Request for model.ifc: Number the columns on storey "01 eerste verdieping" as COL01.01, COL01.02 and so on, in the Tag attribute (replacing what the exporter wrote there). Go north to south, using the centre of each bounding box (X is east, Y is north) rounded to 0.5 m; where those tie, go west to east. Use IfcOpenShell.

First a look at what the model holds.

```python
import ifcopenshell
import ifcopenshell.util.element
import ifcopenshell.util.placement

model = ifcopenshell.open("model.ifc")
print(model.schema)
storey = next(s for s in model.by_type("IfcBuildingStorey") if s.Name == "01 eerste verdieping")
columns = [e for e in ifcopenshell.util.element.get_decomposition(storey) if e.is_a("IfcColumn")]
for e in sorted(columns, key=lambda e: e.id()):
    origin = ifcopenshell.util.placement.get_local_placement(e.ObjectPlacement)[:3, 3]
    print(e.id(), e.Tag, e.Name, origin.round(2) + 0.0, sep=" | ")
```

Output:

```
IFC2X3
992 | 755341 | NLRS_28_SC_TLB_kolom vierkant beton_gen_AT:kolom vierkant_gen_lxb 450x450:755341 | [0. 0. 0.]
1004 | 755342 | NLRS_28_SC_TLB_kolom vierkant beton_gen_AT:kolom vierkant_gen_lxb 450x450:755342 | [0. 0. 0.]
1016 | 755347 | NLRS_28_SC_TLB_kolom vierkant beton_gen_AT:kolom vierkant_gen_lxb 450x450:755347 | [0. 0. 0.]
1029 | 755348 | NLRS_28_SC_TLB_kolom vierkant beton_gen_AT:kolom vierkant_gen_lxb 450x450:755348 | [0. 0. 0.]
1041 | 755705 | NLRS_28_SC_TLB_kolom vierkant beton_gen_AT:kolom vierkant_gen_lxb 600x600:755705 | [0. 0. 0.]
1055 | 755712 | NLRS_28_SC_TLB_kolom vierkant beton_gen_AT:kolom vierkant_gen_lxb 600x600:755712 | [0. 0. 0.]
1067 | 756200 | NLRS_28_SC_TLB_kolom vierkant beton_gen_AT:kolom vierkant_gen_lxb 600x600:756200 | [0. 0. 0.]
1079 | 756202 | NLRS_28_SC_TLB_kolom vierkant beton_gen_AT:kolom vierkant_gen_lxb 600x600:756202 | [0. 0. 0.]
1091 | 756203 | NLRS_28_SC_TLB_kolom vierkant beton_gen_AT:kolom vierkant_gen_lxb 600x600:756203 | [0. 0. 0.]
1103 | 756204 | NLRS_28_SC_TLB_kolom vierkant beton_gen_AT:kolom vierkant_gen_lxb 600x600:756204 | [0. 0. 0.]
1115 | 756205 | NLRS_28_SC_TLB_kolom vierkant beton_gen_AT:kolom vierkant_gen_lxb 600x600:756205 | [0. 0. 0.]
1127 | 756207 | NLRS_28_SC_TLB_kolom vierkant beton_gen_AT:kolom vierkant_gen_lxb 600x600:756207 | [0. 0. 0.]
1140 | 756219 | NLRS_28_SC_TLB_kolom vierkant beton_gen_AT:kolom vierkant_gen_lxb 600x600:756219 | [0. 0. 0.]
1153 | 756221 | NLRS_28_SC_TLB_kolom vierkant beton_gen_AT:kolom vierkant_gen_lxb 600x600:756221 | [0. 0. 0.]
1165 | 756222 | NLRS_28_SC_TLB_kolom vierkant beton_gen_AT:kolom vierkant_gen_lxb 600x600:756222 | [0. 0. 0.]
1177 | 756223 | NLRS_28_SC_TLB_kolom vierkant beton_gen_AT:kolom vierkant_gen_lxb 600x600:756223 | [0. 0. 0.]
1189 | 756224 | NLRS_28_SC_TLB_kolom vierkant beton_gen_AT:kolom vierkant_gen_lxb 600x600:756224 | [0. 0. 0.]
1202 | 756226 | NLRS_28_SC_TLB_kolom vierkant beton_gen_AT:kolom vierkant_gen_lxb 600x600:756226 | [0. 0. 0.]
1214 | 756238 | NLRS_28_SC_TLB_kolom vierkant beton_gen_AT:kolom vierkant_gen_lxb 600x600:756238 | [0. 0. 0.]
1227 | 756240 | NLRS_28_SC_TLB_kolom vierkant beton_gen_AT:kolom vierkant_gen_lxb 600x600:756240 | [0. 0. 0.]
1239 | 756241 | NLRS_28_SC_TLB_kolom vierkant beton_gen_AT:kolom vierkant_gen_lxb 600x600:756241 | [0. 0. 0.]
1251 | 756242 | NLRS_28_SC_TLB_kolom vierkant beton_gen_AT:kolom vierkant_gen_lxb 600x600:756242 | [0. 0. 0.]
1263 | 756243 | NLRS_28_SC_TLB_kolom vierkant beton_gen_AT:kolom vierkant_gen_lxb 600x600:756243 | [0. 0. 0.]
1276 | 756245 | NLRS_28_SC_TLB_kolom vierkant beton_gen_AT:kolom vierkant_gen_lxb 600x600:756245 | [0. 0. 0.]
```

```python
import ifcopenshell
import ifcopenshell.geom
import ifcopenshell.util.element
import ifcopenshell.util.shape

model = ifcopenshell.open("model.ifc")
settings = ifcopenshell.geom.settings()
settings.set("use-world-coords", True)


def centre(element):
    shape = ifcopenshell.geom.create_shape(settings, element)
    return ifcopenshell.util.shape.get_bbox_centroid(shape.geometry)


storey = next(s for s in model.by_type("IfcBuildingStorey") if s.Name == "01 eerste verdieping")
columns = [e for e in ifcopenshell.util.element.get_decomposition(storey) if e.is_a("IfcColumn")]

# Insertion points can sit at a corner or the storey origin, so sort by the geometry (in metres).
centres = {e: centre(e) for e in columns}
columns.sort(key=lambda e: (-round(centres[e][1] / 0.5), centres[e][0]))

for i, e in enumerate(columns, start=1):
    number = f"COL01.{i:02d}"
    e.Tag = number
    print(e.id(), number)

model.write("model_rev.ifc")
```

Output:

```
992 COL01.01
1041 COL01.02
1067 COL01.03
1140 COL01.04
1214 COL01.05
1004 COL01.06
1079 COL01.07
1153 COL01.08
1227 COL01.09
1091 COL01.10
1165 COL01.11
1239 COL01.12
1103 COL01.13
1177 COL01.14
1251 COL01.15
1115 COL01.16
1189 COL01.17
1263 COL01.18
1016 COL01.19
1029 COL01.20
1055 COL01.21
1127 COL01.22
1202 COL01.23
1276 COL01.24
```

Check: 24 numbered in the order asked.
